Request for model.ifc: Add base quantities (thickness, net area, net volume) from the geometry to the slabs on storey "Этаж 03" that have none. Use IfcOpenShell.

First a look at what the model holds.

```python
import ifcopenshell
import ifcopenshell.util.element
import ifcopenshell.util.unit

model = ifcopenshell.open("model.ifc")
print(model.schema)
for unit_type in ("LENGTHUNIT", "AREAUNIT", "VOLUMEUNIT"):
    print(unit_type, ifcopenshell.util.unit.calculate_unit_scale(model, unit_type))
storey = next(s for s in model.by_type("IfcBuildingStorey") if s.Name == "Этаж 03")
slabs = [e for e in ifcopenshell.util.element.get_decomposition(storey) if e.is_a("IfcSlab")]
for e in sorted(slabs, key=lambda e: e.id()):
    print(e.id(), e.is_a(), e.Name, list(ifcopenshell.util.element.get_psets(e, qtos_only=True)), sep=" | ")
```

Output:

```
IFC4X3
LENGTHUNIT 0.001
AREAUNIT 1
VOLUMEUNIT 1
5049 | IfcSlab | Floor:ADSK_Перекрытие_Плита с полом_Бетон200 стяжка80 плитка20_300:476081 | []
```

```python
import ifcopenshell
import ifcopenshell.api.pset
import ifcopenshell.geom
import ifcopenshell.util.element
import ifcopenshell.util.shape
import ifcopenshell.util.unit

model = ifcopenshell.open("model.ifc")
unit_scale = ifcopenshell.util.unit.calculate_unit_scale(model)
area_scale = ifcopenshell.util.unit.calculate_unit_scale(model, "AREAUNIT")
volume_scale = ifcopenshell.util.unit.calculate_unit_scale(model, "VOLUMEUNIT")
settings = ifcopenshell.geom.settings()

storey = next(s for s in model.by_type("IfcBuildingStorey") if s.Name == "Этаж 03")
slabs = [e for e in ifcopenshell.util.element.get_decomposition(storey) if e.is_a("IfcSlab")]

for e in sorted(slabs, key=lambda e: e.id()):
    if ifcopenshell.util.element.get_psets(e, qtos_only=True, should_inherit=False):
        continue
    # Geometry comes back in metres, in the element's own axes.
    shape = ifcopenshell.geom.create_shape(settings, e)
    values = {
        "Width": ifcopenshell.util.shape.get_z(shape.geometry) / unit_scale,
        "NetArea": ifcopenshell.util.shape.get_footprint_area(shape.geometry) / area_scale,
        "NetVolume": ifcopenshell.util.shape.get_volume(shape.geometry) / volume_scale,
    }
    qto = ifcopenshell.api.pset.add_qto(model, product=e, name="Qto_SlabBaseQuantities")
    ifcopenshell.api.pset.edit_qto(model, qto=qto, properties=values)
    print(e.id(), {k: round(v, 3) for k, v in values.items()})

model.write("model-out.ifc")
```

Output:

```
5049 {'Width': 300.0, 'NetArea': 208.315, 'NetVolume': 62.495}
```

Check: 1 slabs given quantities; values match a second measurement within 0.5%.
